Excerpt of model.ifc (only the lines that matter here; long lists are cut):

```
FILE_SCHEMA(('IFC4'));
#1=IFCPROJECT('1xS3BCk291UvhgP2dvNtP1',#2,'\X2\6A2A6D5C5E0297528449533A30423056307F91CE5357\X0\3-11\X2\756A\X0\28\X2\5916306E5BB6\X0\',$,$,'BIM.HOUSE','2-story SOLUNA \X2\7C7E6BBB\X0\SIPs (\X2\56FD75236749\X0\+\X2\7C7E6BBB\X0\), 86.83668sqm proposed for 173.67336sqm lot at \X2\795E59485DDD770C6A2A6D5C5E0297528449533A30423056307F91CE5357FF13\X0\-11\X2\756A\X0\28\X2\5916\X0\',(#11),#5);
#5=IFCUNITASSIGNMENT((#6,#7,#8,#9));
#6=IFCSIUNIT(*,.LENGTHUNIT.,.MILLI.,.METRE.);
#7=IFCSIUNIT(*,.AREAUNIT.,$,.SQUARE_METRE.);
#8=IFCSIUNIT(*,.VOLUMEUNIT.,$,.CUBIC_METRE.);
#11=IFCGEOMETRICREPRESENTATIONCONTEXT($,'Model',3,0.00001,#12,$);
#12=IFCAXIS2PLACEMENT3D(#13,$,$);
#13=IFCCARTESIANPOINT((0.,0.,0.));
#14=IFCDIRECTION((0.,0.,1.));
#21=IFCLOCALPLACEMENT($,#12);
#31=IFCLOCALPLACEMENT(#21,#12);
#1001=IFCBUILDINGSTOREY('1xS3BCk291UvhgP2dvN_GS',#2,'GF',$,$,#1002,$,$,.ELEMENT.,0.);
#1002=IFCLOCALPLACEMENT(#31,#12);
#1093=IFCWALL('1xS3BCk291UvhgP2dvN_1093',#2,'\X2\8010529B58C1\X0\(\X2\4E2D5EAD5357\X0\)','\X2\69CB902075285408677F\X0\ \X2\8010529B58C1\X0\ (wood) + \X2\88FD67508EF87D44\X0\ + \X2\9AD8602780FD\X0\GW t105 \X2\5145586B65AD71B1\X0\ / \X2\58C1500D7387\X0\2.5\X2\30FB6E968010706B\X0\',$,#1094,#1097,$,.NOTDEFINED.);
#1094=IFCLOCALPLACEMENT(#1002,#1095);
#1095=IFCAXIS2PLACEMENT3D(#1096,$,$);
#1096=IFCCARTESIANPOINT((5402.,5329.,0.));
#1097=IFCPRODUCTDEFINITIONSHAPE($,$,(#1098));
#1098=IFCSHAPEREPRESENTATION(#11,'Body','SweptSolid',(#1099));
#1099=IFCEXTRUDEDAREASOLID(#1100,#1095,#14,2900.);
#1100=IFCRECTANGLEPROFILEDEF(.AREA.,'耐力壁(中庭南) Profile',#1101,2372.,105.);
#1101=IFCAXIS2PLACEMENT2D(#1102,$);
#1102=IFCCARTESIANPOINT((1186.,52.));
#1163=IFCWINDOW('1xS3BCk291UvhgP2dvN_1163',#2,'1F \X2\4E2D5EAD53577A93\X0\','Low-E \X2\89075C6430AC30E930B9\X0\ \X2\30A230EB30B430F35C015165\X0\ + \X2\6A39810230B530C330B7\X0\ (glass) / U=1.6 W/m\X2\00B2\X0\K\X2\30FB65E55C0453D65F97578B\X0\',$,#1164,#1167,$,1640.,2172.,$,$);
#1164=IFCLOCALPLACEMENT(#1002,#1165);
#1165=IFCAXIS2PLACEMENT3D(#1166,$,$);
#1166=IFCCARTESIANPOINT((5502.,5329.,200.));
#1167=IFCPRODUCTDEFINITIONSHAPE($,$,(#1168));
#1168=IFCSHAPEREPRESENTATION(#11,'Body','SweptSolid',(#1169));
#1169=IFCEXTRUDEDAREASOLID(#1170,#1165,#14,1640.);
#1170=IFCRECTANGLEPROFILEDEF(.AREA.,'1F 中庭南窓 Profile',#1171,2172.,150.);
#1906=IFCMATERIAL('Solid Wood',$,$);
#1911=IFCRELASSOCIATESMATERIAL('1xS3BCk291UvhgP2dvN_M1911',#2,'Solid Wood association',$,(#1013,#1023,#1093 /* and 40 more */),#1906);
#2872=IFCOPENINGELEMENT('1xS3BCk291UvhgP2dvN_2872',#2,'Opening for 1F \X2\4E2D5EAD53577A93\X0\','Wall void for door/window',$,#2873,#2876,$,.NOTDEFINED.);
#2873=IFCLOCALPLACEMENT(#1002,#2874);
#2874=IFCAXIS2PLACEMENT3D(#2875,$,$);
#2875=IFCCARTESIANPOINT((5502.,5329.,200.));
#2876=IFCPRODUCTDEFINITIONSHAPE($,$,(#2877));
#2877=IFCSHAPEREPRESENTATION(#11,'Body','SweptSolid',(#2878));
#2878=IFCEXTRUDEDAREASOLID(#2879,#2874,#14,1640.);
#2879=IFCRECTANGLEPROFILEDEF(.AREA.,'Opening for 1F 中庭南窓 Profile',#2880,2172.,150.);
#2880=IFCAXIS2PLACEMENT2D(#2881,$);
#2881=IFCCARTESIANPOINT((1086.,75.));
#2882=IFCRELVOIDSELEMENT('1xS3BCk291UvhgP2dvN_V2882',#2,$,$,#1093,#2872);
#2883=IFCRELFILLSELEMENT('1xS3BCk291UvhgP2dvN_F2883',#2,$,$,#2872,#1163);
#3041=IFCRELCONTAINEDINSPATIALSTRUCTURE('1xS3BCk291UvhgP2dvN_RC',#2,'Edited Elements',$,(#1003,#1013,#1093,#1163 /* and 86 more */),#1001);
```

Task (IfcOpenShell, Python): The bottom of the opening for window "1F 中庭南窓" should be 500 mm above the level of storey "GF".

```python
import numpy as np
import ifcopenshell
import ifcopenshell.api.geometry
import ifcopenshell.geom
import ifcopenshell.util.element
import ifcopenshell.util.placement
import ifcopenshell.util.shape
import ifcopenshell.util.unit

model = ifcopenshell.open("model.ifc")
unit_scale = ifcopenshell.util.unit.calculate_unit_scale(model)

window = model.by_id(1163)
opening = window.FillsVoids[0].RelatingOpeningElement
storey = ifcopenshell.util.element.get_container(window, ifc_class="IfcBuildingStorey")
level = ifcopenshell.util.placement.get_local_placement(storey.ObjectPlacement)[2, 3]

# The opening's origin need not be at the sill, so measure its lowest point.
shape = ifcopenshell.geom.create_shape(ifcopenshell.geom.settings(), opening)
bottom = ifcopenshell.util.shape.get_shape_bottom_elevation(shape, shape.geometry) / unit_scale
dz = level + 500.0 - bottom

shift = np.array([0.0, 0.0, dz])
# The window is not placed relative to its opening, so move both.
for product in (opening, window):
    matrix = ifcopenshell.util.placement.get_local_placement(product.ObjectPlacement)
    matrix[:3, 3] += shift
    ifcopenshell.api.geometry.edit_object_placement(model, product=product, matrix=matrix, is_si=False)

print(f"moved by {dz * unit_scale:+.3f} m")

model.write("model_edited.ifc")
```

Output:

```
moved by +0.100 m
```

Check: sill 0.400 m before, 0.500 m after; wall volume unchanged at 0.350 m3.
